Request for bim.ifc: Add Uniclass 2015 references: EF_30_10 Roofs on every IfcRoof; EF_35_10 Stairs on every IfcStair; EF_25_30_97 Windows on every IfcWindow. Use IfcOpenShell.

First a look at what the model holds.

```python
import ifcopenshell

model = ifcopenshell.open("bim.ifc")
print(model.schema)
print("classifications:", [c.Name for c in model.by_type("IfcClassification")])
for ifc_class in ("IfcDoor", "IfcRoof", "IfcStair", "IfcWall", "IfcWindow"):
    print(ifc_class, len(model.by_type(ifc_class)))
```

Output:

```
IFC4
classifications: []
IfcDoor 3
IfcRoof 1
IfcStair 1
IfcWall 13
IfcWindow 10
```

```python
import ifcopenshell
import ifcopenshell.api.classification

model = ifcopenshell.open("bim.ifc")

system = ifcopenshell.api.classification.add_classification(model, classification="Uniclass 2015")

codes = {
    "IfcRoof": ("EF_30_10", "Roofs"),
    "IfcStair": ("EF_35_10", "Stairs"),
    "IfcWindow": ("EF_25_30_97", "Windows"),
}
for ifc_class, (code, name) in codes.items():
    products = model.by_type(ifc_class)
    ifcopenshell.api.classification.add_reference(
        model, products=products, classification=system, identification=code, name=name
    )
    print(code, len(products))

model.write("bim_rev.ifc")
```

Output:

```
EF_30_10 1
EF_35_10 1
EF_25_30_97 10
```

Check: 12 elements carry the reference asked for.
